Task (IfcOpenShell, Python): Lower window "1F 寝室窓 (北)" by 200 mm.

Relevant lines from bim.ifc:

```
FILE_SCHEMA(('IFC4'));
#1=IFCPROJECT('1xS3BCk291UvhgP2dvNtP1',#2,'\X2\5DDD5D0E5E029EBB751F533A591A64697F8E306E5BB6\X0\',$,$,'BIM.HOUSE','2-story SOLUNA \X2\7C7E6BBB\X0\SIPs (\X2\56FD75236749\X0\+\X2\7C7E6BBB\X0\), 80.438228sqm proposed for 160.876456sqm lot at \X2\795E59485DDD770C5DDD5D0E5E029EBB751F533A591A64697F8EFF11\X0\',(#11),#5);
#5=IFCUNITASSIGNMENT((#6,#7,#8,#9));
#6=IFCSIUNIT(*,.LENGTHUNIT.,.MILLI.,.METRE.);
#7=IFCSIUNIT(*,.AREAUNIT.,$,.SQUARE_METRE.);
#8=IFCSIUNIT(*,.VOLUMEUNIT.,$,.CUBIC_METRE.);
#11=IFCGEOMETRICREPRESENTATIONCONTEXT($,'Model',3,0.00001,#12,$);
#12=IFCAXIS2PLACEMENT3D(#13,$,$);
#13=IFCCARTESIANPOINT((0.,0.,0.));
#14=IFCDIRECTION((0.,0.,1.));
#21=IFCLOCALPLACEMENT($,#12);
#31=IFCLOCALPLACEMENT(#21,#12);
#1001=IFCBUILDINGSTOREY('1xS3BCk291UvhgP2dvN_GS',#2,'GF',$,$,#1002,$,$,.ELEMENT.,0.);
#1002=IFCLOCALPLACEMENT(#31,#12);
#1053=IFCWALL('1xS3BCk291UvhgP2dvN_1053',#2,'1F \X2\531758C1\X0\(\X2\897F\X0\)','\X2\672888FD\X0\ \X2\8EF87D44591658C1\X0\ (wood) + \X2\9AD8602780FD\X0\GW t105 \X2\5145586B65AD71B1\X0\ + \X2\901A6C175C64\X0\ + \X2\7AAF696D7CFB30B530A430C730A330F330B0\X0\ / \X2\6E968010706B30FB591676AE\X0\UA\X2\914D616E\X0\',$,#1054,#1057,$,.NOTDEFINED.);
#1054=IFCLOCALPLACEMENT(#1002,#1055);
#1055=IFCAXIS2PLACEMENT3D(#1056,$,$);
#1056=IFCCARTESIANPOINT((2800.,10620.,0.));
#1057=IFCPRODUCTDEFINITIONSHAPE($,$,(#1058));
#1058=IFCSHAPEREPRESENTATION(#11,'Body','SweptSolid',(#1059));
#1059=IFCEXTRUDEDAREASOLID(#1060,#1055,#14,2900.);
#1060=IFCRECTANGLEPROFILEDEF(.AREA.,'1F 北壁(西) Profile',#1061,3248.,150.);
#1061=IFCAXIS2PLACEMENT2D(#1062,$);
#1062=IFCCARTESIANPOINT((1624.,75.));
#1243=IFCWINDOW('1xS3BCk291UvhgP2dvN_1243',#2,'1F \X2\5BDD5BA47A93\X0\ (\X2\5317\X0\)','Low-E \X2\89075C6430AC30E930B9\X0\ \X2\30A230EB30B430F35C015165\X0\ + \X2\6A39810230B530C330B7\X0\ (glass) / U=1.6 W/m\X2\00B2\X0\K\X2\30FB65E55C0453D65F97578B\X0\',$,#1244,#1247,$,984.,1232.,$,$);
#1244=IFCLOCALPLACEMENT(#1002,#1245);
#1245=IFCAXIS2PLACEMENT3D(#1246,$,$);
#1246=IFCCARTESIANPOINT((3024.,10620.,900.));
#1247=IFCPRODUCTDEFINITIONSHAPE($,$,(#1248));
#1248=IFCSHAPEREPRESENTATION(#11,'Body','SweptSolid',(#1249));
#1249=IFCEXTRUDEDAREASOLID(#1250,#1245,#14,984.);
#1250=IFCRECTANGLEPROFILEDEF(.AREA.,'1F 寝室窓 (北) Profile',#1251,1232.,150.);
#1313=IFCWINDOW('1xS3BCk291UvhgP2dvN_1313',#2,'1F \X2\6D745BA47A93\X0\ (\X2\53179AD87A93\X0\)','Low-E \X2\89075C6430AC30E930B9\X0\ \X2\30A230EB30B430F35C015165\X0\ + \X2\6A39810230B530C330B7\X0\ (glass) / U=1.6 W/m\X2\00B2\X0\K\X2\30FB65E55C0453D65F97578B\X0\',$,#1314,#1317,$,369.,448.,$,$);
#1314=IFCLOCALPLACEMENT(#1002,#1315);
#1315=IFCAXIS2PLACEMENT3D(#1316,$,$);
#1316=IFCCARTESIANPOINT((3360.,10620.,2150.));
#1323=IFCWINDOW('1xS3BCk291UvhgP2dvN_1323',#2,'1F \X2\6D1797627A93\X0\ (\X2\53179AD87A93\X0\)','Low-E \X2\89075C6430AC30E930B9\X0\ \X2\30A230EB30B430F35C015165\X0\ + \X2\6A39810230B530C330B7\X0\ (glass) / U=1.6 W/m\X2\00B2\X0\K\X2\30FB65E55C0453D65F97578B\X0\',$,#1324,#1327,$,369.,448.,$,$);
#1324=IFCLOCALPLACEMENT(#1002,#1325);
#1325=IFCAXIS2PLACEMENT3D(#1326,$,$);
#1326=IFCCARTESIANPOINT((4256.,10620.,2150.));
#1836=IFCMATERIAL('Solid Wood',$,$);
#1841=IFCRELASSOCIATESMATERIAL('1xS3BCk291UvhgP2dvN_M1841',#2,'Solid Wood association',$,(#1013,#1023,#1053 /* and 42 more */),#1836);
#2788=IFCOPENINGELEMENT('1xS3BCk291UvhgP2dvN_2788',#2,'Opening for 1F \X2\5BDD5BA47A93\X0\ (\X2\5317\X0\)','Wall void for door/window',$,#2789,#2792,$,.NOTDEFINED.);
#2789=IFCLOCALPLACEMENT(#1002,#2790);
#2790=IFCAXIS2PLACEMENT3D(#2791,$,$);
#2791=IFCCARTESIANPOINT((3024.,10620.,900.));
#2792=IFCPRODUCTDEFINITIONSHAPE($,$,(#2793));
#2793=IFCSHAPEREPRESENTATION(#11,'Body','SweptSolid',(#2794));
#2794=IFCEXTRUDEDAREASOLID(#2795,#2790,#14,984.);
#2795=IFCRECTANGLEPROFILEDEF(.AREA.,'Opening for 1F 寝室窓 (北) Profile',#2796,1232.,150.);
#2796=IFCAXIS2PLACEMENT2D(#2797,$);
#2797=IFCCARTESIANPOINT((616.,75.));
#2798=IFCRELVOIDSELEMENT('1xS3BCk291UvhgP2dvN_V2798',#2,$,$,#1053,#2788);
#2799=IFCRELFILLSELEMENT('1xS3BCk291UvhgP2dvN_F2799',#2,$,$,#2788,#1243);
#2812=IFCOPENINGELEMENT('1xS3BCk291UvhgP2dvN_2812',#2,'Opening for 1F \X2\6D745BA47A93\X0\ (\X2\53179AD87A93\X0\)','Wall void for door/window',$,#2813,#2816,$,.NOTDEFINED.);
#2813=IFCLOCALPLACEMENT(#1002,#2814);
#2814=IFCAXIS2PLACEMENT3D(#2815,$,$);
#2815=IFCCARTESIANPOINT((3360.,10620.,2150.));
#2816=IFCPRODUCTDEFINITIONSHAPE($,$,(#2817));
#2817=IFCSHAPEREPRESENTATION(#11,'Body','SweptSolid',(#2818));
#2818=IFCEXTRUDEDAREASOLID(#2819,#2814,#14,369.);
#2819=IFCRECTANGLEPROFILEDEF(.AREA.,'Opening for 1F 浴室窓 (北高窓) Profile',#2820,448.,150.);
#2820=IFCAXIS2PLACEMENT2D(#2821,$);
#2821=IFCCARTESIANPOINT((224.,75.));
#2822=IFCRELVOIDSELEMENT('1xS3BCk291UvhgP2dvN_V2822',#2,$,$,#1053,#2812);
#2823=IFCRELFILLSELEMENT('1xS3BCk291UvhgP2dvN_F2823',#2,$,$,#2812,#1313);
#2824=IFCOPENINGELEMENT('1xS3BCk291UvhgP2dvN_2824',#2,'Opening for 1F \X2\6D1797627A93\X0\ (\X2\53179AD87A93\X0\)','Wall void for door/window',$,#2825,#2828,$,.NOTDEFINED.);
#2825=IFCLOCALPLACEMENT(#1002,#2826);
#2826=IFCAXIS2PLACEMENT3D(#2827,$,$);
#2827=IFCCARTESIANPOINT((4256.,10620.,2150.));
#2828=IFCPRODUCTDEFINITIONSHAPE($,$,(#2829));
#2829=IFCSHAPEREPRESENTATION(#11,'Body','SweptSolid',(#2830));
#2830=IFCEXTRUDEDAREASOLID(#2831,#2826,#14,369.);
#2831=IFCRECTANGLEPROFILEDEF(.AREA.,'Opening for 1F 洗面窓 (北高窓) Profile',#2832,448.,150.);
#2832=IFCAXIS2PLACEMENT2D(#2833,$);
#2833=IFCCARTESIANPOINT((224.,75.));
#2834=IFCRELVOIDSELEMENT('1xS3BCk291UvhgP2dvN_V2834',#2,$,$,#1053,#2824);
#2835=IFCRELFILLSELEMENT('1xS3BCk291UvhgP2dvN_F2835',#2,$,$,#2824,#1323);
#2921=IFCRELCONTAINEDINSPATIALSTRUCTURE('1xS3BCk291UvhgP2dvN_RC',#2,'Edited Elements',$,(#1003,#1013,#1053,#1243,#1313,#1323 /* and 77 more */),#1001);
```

```python
import numpy as np
import ifcopenshell
import ifcopenshell.api.geometry
import ifcopenshell.util.placement
import ifcopenshell.util.unit

model = ifcopenshell.open("bim.ifc")
unit_scale = ifcopenshell.util.unit.calculate_unit_scale(model)

window = model.by_guid("1xS3BCk291UvhgP2dvN_1243")
opening = window.FillsVoids[0].RelatingOpeningElement
dz = -0.2 / unit_scale

shift = np.array([0.0, 0.0, dz])
# The window is not placed relative to its opening, so move both.
for product in (opening, window):
    matrix = ifcopenshell.util.placement.get_local_placement(product.ObjectPlacement)
    matrix[:3, 3] += shift
    ifcopenshell.api.geometry.edit_object_placement(model, product=product, matrix=matrix, is_si=False)

print(f"moved by {dz * unit_scale:+.3f} m")

model.write("bim_edited.ifc")
```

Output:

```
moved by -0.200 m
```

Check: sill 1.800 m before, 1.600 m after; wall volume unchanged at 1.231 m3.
